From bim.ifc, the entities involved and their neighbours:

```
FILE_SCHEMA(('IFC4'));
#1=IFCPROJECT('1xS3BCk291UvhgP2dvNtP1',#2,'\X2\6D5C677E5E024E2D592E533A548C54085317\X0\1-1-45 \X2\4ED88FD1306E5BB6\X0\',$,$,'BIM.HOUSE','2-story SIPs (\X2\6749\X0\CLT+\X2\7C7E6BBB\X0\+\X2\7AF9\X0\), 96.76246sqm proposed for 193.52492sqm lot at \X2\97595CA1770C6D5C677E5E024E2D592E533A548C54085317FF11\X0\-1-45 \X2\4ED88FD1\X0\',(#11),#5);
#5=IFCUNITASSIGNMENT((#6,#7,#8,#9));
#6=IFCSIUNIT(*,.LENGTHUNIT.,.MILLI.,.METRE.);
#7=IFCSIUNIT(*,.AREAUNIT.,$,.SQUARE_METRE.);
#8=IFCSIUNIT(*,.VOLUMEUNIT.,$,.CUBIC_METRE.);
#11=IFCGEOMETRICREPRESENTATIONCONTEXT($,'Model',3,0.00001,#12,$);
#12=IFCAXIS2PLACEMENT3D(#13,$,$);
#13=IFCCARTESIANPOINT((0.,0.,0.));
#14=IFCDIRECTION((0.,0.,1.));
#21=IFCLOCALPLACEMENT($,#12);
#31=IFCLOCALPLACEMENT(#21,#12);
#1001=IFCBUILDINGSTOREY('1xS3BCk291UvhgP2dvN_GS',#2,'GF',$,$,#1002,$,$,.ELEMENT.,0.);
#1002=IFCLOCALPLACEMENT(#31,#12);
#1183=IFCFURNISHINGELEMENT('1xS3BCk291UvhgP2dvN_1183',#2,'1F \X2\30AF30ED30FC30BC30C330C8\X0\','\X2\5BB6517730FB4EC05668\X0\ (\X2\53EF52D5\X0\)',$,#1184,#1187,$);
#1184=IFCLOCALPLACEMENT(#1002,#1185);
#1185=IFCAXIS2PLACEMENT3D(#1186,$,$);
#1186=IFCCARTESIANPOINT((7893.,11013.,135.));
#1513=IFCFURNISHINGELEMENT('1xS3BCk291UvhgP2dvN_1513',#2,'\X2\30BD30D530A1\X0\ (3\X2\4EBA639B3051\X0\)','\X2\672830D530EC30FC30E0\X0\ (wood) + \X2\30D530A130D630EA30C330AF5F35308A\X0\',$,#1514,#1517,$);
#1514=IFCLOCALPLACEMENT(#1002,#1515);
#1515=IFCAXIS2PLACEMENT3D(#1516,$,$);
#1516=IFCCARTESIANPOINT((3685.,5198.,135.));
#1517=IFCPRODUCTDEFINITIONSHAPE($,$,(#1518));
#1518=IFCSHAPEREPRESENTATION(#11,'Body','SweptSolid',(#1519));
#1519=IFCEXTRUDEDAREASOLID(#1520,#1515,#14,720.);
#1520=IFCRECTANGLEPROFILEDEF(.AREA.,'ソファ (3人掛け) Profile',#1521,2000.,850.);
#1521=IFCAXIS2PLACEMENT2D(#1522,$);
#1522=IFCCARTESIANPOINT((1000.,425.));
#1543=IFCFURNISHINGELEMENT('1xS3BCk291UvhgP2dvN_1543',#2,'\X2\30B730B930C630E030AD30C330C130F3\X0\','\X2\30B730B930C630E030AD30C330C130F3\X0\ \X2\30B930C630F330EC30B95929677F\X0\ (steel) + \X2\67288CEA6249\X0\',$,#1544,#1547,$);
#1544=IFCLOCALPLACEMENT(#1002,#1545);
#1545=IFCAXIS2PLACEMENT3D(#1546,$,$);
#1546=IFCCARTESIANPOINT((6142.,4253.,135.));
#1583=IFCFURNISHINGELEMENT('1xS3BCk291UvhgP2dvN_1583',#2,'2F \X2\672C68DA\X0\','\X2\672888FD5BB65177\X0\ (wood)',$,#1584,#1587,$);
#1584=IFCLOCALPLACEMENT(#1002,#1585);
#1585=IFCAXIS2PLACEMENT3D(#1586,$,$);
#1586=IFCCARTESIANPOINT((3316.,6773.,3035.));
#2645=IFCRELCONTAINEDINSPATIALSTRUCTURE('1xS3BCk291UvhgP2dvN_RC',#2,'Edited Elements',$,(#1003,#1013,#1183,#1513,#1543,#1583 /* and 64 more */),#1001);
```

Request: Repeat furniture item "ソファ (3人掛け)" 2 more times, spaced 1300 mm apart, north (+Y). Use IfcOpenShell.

```python
import numpy as np
import ifcopenshell
import ifcopenshell.api.geometry
import ifcopenshell.api.root
import ifcopenshell.util.element
import ifcopenshell.util.placement
import ifcopenshell.util.unit

model = ifcopenshell.open("bim.ifc")
unit_scale = ifcopenshell.util.unit.calculate_unit_scale(model)


def reuse_history(source, copy):
    """copy_class also copies each property set's owner history, people and application; keep the originals."""
    for rel in copy.IsDefinedBy:
        if rel.is_a("IfcRelDefinesByProperties") and (history := rel.RelatingPropertyDefinition.OwnerHistory):
            rel.RelatingPropertyDefinition.OwnerHistory = source.OwnerHistory
            ifcopenshell.util.element.remove_deep2(model, history)


source = model.by_guid("1xS3BCk291UvhgP2dvN_1513")
base = ifcopenshell.util.placement.get_local_placement(source.ObjectPlacement)
step = np.array([0.0, 1.0, 0.0]) * 1.3 / unit_scale

for i in range(1, 3):
    copy = ifcopenshell.api.root.copy_class(model, product=source)
    copy.Representation = ifcopenshell.util.element.copy_deep(
        model, source.Representation, exclude=["IfcGeometricRepresentationContext", "IfcRepresentationMap"]
    )
    reuse_history(source, copy)
    matrix = base.copy()
    matrix[:3, 3] += i * step
    print("added at", matrix[:3, 3].round(3) + 0.0)
    ifcopenshell.api.geometry.edit_object_placement(model, product=copy, matrix=matrix, is_si=False)

model.write("bim_rev.ifc")
```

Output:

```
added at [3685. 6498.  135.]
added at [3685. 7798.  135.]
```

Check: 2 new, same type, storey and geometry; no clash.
